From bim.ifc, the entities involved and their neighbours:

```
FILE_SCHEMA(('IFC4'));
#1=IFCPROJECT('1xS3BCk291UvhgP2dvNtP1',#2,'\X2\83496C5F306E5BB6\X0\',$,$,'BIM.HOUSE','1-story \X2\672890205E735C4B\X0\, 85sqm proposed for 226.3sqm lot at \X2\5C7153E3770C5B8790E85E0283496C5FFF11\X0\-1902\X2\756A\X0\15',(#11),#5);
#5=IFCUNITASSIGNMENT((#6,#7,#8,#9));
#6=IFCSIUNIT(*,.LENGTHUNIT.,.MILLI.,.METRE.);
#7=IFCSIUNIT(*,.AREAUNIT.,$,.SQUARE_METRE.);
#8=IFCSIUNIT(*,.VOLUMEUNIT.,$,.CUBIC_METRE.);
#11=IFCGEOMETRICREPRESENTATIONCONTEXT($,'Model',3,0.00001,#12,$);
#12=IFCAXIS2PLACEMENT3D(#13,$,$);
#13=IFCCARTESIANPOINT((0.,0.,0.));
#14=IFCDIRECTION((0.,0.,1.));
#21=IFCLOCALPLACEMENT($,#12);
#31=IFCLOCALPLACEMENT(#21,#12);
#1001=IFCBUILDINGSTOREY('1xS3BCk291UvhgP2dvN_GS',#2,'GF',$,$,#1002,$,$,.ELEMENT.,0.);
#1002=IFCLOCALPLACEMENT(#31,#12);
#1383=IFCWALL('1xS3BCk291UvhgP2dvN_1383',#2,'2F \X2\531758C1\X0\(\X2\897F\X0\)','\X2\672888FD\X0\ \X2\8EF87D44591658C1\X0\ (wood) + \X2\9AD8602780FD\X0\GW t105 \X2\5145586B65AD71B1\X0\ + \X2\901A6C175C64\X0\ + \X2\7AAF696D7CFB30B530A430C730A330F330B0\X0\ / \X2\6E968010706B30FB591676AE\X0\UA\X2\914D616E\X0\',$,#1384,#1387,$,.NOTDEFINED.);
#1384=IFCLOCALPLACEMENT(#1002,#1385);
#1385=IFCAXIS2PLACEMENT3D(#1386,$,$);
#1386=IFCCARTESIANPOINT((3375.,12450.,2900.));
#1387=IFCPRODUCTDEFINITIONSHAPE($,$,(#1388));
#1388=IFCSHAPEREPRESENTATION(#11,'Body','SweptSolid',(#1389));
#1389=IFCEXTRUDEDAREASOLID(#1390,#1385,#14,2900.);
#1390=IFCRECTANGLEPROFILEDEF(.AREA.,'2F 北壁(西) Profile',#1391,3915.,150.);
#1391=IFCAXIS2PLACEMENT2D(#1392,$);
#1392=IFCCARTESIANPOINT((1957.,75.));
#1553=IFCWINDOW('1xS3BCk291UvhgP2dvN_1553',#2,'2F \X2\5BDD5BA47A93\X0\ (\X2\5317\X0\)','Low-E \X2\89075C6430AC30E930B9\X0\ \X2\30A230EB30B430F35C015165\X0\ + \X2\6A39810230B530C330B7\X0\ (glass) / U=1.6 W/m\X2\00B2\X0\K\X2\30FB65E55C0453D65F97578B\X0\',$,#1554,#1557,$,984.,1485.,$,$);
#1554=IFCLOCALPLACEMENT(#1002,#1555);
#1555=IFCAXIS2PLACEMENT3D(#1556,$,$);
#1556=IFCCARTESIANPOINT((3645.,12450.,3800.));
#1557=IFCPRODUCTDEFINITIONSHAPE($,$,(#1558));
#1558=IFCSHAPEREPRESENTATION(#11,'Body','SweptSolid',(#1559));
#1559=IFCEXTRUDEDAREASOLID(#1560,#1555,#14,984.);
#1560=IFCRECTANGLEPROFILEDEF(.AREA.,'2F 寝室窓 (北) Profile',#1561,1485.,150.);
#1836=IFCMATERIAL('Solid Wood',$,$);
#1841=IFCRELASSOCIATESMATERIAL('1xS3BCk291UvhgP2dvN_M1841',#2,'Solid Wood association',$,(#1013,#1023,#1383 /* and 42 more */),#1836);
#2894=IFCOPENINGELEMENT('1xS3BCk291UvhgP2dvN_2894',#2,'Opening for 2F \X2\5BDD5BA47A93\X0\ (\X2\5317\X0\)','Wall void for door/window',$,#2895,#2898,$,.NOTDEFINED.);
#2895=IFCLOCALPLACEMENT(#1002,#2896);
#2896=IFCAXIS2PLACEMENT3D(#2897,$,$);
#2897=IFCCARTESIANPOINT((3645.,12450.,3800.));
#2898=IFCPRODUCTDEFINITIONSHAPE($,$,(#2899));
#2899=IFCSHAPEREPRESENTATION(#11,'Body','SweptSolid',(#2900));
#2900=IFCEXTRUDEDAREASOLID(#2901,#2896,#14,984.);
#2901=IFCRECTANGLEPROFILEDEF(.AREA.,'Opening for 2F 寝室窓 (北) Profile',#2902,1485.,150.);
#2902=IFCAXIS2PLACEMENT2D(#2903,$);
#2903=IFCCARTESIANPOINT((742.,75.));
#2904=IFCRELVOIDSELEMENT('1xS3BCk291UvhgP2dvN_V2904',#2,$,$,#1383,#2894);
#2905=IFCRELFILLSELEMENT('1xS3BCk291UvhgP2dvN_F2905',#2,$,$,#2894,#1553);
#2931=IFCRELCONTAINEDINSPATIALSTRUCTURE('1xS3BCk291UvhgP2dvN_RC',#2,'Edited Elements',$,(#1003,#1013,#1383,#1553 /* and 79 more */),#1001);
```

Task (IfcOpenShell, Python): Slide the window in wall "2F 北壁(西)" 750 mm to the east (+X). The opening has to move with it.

```python
import ifcopenshell
import ifcopenshell.api.geometry
import ifcopenshell.util.placement
import ifcopenshell.util.unit

model = ifcopenshell.open("bim.ifc")
unit_scale = ifcopenshell.util.unit.calculate_unit_scale(model)

window = model.by_guid("1xS3BCk291UvhgP2dvN_1553")
opening = window.FillsVoids[0].RelatingOpeningElement
wall = opening.VoidsElements[0].RelatingBuildingElement

wall_matrix = ifcopenshell.util.placement.get_local_placement(wall.ObjectPlacement)
shift = wall_matrix[:3, 0] * 0.75 / unit_scale
before = ifcopenshell.util.placement.get_local_placement(window.ObjectPlacement)[:3, 3].copy()

# The window is not placed relative to its opening, so move both.
for product in (opening, window):
    matrix = ifcopenshell.util.placement.get_local_placement(product.ObjectPlacement)
    matrix[:3, 3] += shift
    ifcopenshell.api.geometry.edit_object_placement(model, product=product, matrix=matrix, is_si=False)

after = ifcopenshell.util.placement.get_local_placement(window.ObjectPlacement)[:3, 3]
print("window moved by", (after - before).round(3) + 0.0)

model.write("bim_edited.ifc")
```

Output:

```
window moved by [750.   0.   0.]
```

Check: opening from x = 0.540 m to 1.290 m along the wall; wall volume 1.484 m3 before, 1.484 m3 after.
